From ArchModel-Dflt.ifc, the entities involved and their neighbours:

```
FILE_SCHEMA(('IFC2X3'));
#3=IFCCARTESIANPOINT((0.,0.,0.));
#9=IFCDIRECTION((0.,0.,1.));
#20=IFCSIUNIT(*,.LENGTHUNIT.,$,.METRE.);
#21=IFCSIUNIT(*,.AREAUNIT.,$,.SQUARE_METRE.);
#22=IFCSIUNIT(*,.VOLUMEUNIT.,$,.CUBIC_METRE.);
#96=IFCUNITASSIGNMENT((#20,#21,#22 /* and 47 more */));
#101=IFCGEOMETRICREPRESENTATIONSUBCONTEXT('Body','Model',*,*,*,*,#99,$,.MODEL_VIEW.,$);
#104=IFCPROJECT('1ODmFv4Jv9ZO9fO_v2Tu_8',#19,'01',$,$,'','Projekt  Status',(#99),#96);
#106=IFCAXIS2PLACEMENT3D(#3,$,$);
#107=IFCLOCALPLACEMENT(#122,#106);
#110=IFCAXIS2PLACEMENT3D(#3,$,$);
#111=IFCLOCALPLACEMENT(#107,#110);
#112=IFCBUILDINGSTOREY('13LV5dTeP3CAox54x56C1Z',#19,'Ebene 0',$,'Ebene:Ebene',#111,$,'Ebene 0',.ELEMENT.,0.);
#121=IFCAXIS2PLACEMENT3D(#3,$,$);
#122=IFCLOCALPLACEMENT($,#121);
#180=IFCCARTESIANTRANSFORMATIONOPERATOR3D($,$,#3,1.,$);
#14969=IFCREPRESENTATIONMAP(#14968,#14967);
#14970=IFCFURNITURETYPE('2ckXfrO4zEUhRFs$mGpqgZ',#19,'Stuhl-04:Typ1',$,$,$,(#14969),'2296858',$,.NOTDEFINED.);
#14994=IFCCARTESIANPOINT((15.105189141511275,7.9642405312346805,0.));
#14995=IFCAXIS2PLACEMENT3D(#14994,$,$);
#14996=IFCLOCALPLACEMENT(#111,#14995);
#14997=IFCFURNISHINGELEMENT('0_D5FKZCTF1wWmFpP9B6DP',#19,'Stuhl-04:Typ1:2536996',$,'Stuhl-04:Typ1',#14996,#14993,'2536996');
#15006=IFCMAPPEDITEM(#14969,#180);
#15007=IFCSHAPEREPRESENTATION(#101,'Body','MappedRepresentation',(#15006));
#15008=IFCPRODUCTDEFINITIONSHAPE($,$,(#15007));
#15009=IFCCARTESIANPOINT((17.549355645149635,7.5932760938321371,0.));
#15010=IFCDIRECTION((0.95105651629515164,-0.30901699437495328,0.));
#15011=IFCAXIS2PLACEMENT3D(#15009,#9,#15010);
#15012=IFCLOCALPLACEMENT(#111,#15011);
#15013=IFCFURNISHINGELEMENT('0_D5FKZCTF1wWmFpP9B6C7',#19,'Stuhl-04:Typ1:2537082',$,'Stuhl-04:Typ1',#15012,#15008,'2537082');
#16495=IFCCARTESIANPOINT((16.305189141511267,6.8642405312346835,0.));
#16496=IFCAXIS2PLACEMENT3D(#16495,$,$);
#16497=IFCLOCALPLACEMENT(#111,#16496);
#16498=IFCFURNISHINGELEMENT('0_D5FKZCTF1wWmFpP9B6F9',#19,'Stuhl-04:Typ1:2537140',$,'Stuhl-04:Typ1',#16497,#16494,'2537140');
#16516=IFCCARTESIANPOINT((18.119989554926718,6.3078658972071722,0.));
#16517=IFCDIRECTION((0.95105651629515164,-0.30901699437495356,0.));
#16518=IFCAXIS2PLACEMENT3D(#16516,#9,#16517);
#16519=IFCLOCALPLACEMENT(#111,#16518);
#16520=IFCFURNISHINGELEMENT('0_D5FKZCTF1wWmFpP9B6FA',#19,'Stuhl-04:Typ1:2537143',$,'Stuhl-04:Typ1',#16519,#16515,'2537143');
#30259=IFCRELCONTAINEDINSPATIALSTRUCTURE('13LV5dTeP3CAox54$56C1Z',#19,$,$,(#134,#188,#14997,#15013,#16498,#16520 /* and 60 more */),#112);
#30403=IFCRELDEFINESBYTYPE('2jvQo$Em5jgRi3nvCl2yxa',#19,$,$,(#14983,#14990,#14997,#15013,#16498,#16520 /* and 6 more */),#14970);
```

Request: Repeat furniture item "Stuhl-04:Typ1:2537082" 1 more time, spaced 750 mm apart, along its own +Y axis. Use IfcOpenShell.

```python
import ifcopenshell
import ifcopenshell.api.geometry
import ifcopenshell.api.root
import ifcopenshell.util.element
import ifcopenshell.util.placement
import ifcopenshell.util.unit

model = ifcopenshell.open("ArchModel-Dflt.ifc")
unit_scale = ifcopenshell.util.unit.calculate_unit_scale(model)

source = model.by_guid("0_D5FKZCTF1wWmFpP9B6C7")
base = ifcopenshell.util.placement.get_local_placement(source.ObjectPlacement)
step = base[:3, 1] * 0.75 / unit_scale

for i in range(1, 2):
    copy = ifcopenshell.api.root.copy_class(model, product=source)
    copy.Representation = ifcopenshell.util.element.copy_deep(
        model, source.Representation, exclude=["IfcGeometricRepresentationContext", "IfcRepresentationMap"]
    )
    copy.Name = "Stuhl-04:Typ1"
    copy.Tag = None
    matrix = base.copy()
    matrix[:3, 3] += i * step
    print("added at", matrix[:3, 3].round(3) + 0.0)
    ifcopenshell.api.geometry.edit_object_placement(model, product=copy, matrix=matrix, is_si=False)

model.write("ArchModel-Dflt-out.ifc")
```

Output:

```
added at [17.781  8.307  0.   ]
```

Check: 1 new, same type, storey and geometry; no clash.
